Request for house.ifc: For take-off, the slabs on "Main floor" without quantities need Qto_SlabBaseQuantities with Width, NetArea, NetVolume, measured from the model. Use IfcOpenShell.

First a look at what the model holds.

```python
import ifcopenshell
import ifcopenshell.util.element
import ifcopenshell.util.unit

model = ifcopenshell.open("house.ifc")
print(model.schema)
for unit_type in ("LENGTHUNIT", "AREAUNIT", "VOLUMEUNIT"):
    print(unit_type, ifcopenshell.util.unit.calculate_unit_scale(model, unit_type))
storey = next(s for s in model.by_type("IfcBuildingStorey") if s.Name == "Main floor")
slabs = [e for e in ifcopenshell.util.element.get_decomposition(storey) if e.is_a("IfcSlab")]
for e in sorted(slabs, key=lambda e: e.id()):
    print(e.id(), e.is_a(), e.Name, list(ifcopenshell.util.element.get_psets(e, qtos_only=True)), sep=" | ")
```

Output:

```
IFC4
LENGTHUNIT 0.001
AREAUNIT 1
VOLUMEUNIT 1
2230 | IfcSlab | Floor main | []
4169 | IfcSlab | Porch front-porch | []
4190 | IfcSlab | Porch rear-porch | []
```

```python
import ifcopenshell
import ifcopenshell.api.pset
import ifcopenshell.geom
import ifcopenshell.util.element
import ifcopenshell.util.shape
import ifcopenshell.util.unit

model = ifcopenshell.open("house.ifc")
unit_scale = ifcopenshell.util.unit.calculate_unit_scale(model)
area_scale = ifcopenshell.util.unit.calculate_unit_scale(model, "AREAUNIT")
volume_scale = ifcopenshell.util.unit.calculate_unit_scale(model, "VOLUMEUNIT")
settings = ifcopenshell.geom.settings()

storey = next(s for s in model.by_type("IfcBuildingStorey") if s.Name == "Main floor")
slabs = [e for e in ifcopenshell.util.element.get_decomposition(storey) if e.is_a("IfcSlab")]

for e in sorted(slabs, key=lambda e: e.id()):
    if ifcopenshell.util.element.get_psets(e, qtos_only=True, should_inherit=False):
        continue
    # Geometry comes back in metres, in the element's own axes.
    shape = ifcopenshell.geom.create_shape(settings, e)
    values = {
        "Width": ifcopenshell.util.shape.get_z(shape.geometry) / unit_scale,
        "NetArea": ifcopenshell.util.shape.get_footprint_area(shape.geometry) / area_scale,
        "NetVolume": ifcopenshell.util.shape.get_volume(shape.geometry) / volume_scale,
    }
    qto = ifcopenshell.api.pset.add_qto(model, product=e, name="Qto_SlabBaseQuantities")
    ifcopenshell.api.pset.edit_qto(model, qto=qto, properties=values)
    print(e.id(), {k: round(v, 3) for k, v in values.items()})

model.write("house-out.ifc")
```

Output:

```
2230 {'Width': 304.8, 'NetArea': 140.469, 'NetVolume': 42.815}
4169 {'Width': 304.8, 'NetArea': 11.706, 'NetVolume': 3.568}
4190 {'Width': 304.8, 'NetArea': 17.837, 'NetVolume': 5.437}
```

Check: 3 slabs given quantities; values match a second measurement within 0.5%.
